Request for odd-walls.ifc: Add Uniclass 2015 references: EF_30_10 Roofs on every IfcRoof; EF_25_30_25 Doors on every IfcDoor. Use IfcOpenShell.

First a look at what the model holds.

```python
import ifcopenshell

model = ifcopenshell.open("odd-walls.ifc")
print(model.schema)
print("classifications:", [c.Name for c in model.by_type("IfcClassification")])
for ifc_class in ("IfcDoor", "IfcRoof", "IfcStair", "IfcWall", "IfcWindow"):
    print(ifc_class, len(model.by_type(ifc_class)))
```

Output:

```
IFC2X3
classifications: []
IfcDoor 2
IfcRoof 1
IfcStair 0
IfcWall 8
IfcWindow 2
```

```python
import ifcopenshell
import ifcopenshell.api.classification

model = ifcopenshell.open("odd-walls.ifc")

# IFC2X3 requires Source and Edition and has no link from the project to the system.
system = model.create_entity("IfcClassification", Source="NBS", Edition="2015", Name="Uniclass 2015")

codes = {
    "IfcRoof": ("EF_30_10", "Roofs"),
    "IfcDoor": ("EF_25_30_25", "Doors"),
}
for ifc_class, (code, name) in codes.items():
    products = model.by_type(ifc_class)
    ifcopenshell.api.classification.add_reference(
        model, products=products, classification=system, identification=code, name=name
    )
    print(code, len(products))

model.write("odd-walls-out.ifc")
```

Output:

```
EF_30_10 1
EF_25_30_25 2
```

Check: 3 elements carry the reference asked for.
